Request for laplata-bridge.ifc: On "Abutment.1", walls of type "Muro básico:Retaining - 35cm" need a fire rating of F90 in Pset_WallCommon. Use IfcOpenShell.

First a look at what the model holds.

```python
import ifcopenshell
import ifcopenshell.util.element

model = ifcopenshell.open("laplata-bridge.ifc")
print(model.schema)
storey = next(s for s in model.by_type("IfcBuildingStorey") if s.Name == "Abutment.1")
walls = [e for e in ifcopenshell.util.element.get_decomposition(storey) if e.is_a("IfcWall")]
seen = {}
for e in walls:
    element_type = ifcopenshell.util.element.get_type(e)
    key = (element_type.Name if element_type != e and element_type else None, ifcopenshell.util.element.get_pset(e, "Pset_WallCommon", "FireRating"))
    seen[key] = seen.get(key, 0) + 1
for (name, value), count in sorted(seen.items(), key=str):
    print(count, "x", name, "|", value)
```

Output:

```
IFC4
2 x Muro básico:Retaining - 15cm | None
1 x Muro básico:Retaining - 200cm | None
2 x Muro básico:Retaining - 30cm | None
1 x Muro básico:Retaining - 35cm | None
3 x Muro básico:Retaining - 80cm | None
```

```python
import ifcopenshell
import ifcopenshell.api.pset
import ifcopenshell.util.element

model = ifcopenshell.open("laplata-bridge.ifc")

storey = next(s for s in model.by_type("IfcBuildingStorey") if s.Name == "Abutment.1")
walls = [e for e in ifcopenshell.util.element.get_decomposition(storey) if e.is_a("IfcWall")]

count = 0
for e in walls:
    element_type = ifcopenshell.util.element.get_type(e)
    if element_type in (None, e) or element_type.Name != "Muro básico:Retaining - 35cm":
        continue
    # add_pset returns the element's existing set when there is one.
    pset = ifcopenshell.api.pset.add_pset(model, product=e, name="Pset_WallCommon")
    ifcopenshell.api.pset.edit_pset(model, pset=pset, properties={"FireRating": "F90"})
    count += 1

print(count, "walls updated")

model.write("laplata-bridge-out.ifc")
```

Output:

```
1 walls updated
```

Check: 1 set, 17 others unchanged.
